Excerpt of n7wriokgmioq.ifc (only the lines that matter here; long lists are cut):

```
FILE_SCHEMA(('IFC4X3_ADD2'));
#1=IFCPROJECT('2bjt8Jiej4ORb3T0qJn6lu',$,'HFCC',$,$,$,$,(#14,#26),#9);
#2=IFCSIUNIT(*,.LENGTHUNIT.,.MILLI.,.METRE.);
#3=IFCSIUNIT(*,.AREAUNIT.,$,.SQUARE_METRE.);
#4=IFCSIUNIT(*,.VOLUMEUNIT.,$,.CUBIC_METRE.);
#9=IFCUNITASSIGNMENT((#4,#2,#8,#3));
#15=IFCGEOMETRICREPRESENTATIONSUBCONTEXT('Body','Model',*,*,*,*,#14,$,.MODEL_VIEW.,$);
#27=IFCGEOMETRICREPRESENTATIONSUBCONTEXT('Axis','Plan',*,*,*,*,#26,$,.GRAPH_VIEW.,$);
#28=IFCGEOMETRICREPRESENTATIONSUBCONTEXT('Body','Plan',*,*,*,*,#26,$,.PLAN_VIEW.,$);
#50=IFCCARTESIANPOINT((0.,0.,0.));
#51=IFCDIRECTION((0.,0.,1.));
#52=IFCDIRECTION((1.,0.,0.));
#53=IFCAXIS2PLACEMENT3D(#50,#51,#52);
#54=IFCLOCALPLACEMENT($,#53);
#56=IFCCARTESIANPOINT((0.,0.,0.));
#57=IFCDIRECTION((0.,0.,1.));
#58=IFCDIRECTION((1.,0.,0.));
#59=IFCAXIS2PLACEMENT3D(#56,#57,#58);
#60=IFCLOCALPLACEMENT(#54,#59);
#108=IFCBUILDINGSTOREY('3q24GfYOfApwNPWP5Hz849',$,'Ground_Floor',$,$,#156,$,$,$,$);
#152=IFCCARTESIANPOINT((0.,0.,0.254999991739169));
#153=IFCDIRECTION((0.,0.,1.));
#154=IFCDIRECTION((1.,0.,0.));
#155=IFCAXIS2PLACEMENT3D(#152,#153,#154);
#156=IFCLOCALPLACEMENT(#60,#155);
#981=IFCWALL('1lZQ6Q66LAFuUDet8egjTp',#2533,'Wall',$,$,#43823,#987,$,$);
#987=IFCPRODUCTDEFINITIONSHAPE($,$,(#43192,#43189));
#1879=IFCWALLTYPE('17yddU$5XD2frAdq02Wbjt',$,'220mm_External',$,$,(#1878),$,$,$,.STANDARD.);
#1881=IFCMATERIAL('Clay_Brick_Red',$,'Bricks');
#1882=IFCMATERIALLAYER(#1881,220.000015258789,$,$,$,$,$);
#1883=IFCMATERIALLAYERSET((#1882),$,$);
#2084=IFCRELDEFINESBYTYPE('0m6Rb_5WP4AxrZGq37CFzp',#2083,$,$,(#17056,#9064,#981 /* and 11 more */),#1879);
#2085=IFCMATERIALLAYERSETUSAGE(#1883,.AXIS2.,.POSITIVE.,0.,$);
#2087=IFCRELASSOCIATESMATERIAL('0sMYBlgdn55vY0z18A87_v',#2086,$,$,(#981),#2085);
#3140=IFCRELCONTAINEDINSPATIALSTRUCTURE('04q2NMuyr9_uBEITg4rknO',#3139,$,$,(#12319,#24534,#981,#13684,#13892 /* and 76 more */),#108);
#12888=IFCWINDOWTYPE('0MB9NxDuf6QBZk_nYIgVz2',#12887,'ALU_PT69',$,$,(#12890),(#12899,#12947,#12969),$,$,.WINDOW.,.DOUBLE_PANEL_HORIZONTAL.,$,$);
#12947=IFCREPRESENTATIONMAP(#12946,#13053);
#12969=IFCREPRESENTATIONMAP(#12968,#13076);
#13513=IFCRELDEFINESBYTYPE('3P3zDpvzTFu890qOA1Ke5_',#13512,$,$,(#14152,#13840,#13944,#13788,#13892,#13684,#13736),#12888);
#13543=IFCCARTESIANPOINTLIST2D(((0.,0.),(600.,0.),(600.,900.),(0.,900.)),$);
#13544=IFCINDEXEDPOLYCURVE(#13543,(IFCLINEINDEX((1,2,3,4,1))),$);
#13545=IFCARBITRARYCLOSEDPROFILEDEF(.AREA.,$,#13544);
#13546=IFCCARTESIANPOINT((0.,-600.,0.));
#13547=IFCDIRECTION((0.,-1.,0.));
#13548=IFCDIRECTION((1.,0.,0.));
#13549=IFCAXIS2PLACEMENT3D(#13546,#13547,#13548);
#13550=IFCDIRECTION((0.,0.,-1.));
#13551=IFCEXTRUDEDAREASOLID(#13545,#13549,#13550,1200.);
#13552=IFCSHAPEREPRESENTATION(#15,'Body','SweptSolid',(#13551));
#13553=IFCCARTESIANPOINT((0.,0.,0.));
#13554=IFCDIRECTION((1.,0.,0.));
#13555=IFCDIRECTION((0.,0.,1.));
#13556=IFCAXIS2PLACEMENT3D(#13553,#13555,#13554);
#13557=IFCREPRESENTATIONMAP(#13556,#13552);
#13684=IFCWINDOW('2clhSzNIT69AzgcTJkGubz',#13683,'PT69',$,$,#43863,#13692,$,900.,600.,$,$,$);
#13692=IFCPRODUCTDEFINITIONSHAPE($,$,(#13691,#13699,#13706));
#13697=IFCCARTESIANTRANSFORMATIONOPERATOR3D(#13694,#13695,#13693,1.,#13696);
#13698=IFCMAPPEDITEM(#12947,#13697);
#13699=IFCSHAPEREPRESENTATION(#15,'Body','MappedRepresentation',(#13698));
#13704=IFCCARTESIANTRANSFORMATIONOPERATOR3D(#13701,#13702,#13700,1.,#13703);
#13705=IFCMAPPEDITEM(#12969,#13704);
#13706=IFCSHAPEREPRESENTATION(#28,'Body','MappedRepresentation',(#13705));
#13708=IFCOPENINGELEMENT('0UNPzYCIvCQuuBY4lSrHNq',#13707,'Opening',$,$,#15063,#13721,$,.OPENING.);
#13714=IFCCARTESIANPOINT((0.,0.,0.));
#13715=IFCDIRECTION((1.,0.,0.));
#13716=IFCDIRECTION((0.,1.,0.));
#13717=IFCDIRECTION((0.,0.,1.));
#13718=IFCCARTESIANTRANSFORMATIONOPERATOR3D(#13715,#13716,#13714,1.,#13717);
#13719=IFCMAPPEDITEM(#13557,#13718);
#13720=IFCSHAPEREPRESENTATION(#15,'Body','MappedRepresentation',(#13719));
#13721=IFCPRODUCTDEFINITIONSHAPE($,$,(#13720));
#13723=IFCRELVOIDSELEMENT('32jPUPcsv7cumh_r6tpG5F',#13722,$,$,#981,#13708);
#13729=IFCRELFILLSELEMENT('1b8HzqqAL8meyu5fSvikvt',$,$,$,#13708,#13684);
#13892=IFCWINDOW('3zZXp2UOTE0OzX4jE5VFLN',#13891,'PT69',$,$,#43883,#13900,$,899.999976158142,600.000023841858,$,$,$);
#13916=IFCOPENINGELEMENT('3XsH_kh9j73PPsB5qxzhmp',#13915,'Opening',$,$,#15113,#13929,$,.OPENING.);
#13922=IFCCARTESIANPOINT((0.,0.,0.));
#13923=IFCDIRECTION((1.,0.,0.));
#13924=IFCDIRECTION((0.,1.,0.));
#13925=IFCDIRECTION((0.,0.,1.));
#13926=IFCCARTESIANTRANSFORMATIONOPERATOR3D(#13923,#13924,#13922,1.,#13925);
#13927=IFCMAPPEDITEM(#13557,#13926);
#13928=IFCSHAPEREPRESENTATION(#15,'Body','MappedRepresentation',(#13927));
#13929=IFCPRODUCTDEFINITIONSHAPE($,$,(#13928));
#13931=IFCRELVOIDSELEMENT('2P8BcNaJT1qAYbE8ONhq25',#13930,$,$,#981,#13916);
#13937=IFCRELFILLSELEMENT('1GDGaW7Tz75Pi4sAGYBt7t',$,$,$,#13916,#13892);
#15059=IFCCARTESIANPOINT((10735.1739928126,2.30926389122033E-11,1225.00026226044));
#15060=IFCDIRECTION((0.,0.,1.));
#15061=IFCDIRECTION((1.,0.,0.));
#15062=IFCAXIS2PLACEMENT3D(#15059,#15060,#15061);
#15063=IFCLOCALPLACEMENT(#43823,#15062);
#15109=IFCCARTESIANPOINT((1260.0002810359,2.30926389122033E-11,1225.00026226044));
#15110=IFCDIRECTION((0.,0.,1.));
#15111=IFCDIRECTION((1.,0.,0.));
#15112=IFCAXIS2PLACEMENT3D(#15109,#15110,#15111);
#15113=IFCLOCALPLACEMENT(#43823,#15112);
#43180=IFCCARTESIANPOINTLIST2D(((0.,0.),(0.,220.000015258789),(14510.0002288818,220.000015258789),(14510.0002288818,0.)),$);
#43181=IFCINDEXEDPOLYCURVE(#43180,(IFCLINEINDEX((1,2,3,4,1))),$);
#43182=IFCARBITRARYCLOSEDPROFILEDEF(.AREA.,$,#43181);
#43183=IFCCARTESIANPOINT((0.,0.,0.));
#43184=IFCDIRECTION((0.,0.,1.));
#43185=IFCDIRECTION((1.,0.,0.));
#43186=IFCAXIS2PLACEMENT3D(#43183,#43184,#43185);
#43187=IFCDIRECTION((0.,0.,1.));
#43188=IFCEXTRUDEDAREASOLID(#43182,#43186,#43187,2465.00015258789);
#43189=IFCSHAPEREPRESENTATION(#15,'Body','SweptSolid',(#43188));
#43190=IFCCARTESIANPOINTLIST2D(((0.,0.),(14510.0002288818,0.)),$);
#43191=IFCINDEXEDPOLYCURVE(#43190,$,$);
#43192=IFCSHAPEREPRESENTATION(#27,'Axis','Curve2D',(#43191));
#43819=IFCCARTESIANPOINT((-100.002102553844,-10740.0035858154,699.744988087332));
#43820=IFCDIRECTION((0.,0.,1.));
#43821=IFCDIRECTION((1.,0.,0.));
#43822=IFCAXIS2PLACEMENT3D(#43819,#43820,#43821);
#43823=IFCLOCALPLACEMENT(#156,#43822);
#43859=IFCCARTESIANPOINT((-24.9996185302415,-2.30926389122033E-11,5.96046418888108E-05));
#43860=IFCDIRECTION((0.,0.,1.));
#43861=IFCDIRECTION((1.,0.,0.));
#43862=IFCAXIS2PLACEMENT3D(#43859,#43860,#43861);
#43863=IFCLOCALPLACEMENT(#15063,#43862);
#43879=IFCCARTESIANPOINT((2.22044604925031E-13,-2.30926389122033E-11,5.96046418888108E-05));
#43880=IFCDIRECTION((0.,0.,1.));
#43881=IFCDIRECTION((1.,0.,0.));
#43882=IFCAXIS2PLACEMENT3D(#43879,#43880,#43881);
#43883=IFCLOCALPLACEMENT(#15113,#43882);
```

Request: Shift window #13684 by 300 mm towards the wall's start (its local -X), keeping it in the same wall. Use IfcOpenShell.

```python
import ifcopenshell
import ifcopenshell.api.geometry
import ifcopenshell.util.placement
import ifcopenshell.util.unit

model = ifcopenshell.open("n7wriokgmioq.ifc")
unit_scale = ifcopenshell.util.unit.calculate_unit_scale(model)

window = model.by_guid("2clhSzNIT69AzgcTJkGubz")
opening = window.FillsVoids[0].RelatingOpeningElement
wall = opening.VoidsElements[0].RelatingBuildingElement

wall_matrix = ifcopenshell.util.placement.get_local_placement(wall.ObjectPlacement)
shift = wall_matrix[:3, 0] * -0.3 / unit_scale
before = ifcopenshell.util.placement.get_local_placement(window.ObjectPlacement)[:3, 3].copy()

# The window is placed relative to its opening, so it follows when the opening moves.
matrix = ifcopenshell.util.placement.get_local_placement(opening.ObjectPlacement)
matrix[:3, 3] += shift
ifcopenshell.api.geometry.edit_object_placement(
    model, product=opening, matrix=matrix, is_si=False, should_transform_children=True
)

after = ifcopenshell.util.placement.get_local_placement(window.ObjectPlacement)[:3, 3]
print("window moved by", (after - before).round(3) + 0.0)

model.write("n7wriokgmioq_edited.ifc")
```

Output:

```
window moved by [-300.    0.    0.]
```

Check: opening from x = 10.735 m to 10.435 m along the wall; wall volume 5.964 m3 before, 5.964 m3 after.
